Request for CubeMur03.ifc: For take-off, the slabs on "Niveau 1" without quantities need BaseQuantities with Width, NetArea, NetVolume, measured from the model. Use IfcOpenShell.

First a look at what the model holds.

```python
import ifcopenshell
import ifcopenshell.util.element
import ifcopenshell.util.unit

model = ifcopenshell.open("CubeMur03.ifc")
print(model.schema)
for unit_type in ("LENGTHUNIT", "AREAUNIT", "VOLUMEUNIT"):
    print(unit_type, ifcopenshell.util.unit.calculate_unit_scale(model, unit_type))
storey = next(s for s in model.by_type("IfcBuildingStorey") if s.Name == "Niveau 1")
slabs = [e for e in ifcopenshell.util.element.get_decomposition(storey) if e.is_a("IfcSlab")]
for e in sorted(slabs, key=lambda e: e.id()):
    print(e.id(), e.is_a(), e.Name, list(ifcopenshell.util.element.get_psets(e, qtos_only=True)), sep=" | ")
```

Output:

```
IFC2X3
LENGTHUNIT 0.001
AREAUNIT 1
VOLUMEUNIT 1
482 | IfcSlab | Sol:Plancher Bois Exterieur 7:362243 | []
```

```python
import ifcopenshell
import ifcopenshell.api.pset
import ifcopenshell.geom
import ifcopenshell.util.element
import ifcopenshell.util.shape
import ifcopenshell.util.unit

model = ifcopenshell.open("CubeMur03.ifc")
unit_scale = ifcopenshell.util.unit.calculate_unit_scale(model)
area_scale = ifcopenshell.util.unit.calculate_unit_scale(model, "AREAUNIT")
volume_scale = ifcopenshell.util.unit.calculate_unit_scale(model, "VOLUMEUNIT")
settings = ifcopenshell.geom.settings()

storey = next(s for s in model.by_type("IfcBuildingStorey") if s.Name == "Niveau 1")
slabs = [e for e in ifcopenshell.util.element.get_decomposition(storey) if e.is_a("IfcSlab")]

for e in sorted(slabs, key=lambda e: e.id()):
    if ifcopenshell.util.element.get_psets(e, qtos_only=True, should_inherit=False):
        continue
    # Geometry comes back in metres, in the element's own axes.
    shape = ifcopenshell.geom.create_shape(settings, e)
    values = {
        "Width": ifcopenshell.util.shape.get_z(shape.geometry) / unit_scale,
        "NetArea": ifcopenshell.util.shape.get_footprint_area(shape.geometry) / area_scale,
        "NetVolume": ifcopenshell.util.shape.get_volume(shape.geometry) / volume_scale,
    }
    qto = ifcopenshell.api.pset.add_qto(model, product=e, name="BaseQuantities")
    ifcopenshell.api.pset.edit_qto(model, qto=qto, properties=values)
    print(e.id(), {k: round(v, 3) for k, v in values.items()})

model.write("CubeMur03_rev.ifc")
```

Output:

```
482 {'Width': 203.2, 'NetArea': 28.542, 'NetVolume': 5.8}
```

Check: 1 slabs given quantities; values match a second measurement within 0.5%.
